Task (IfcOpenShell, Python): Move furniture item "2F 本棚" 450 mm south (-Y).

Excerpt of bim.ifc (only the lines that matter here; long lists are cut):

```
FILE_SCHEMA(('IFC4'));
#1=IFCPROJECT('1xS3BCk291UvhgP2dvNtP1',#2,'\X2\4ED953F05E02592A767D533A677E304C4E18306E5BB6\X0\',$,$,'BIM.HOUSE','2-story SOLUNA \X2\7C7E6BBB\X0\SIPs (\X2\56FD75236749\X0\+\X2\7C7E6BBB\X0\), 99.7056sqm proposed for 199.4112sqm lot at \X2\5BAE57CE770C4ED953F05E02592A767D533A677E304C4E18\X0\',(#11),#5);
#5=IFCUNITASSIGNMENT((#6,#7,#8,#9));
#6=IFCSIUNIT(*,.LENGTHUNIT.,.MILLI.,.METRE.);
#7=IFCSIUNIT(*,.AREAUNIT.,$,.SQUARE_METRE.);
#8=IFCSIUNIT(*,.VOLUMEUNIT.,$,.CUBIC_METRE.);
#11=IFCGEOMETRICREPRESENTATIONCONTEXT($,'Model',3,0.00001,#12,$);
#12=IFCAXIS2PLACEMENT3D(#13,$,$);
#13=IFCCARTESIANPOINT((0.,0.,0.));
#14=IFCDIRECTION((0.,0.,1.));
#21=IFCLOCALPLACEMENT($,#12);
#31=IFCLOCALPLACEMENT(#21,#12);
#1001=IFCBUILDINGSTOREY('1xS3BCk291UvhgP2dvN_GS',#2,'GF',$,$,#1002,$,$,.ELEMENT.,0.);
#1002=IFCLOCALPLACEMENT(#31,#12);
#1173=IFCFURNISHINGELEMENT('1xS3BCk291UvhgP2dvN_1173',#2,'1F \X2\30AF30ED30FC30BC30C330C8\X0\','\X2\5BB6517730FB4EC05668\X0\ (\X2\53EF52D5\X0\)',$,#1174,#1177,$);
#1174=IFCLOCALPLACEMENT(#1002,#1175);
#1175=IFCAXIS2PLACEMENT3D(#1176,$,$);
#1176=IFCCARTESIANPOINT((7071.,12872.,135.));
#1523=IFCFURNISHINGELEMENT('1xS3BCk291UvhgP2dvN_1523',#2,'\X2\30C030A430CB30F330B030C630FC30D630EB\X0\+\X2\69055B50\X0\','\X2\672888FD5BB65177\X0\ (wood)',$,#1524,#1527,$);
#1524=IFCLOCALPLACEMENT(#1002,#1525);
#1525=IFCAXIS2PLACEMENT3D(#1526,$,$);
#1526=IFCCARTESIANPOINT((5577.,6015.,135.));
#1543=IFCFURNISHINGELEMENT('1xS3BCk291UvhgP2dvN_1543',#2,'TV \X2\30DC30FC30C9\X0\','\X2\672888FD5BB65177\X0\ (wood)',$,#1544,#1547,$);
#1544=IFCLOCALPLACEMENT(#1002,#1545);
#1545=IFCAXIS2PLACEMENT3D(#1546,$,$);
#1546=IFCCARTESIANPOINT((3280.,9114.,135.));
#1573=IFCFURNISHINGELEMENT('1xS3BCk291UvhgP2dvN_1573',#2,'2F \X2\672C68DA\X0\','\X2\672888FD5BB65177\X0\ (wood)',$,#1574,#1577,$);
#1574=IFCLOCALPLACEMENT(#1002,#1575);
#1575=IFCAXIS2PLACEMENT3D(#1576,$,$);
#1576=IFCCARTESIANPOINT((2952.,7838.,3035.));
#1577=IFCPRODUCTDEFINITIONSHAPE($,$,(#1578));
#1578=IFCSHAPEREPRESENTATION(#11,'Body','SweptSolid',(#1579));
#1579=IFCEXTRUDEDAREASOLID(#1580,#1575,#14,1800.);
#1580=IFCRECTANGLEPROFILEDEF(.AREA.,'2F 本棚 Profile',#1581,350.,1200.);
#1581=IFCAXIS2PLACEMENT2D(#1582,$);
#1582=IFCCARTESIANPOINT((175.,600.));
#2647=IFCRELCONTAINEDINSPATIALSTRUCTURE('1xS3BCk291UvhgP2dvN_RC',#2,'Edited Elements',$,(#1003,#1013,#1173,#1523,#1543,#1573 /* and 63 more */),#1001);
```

```python
import ifcopenshell
import ifcopenshell.api.geometry
import ifcopenshell.util.placement

model = ifcopenshell.open("bim.ifc")

item = model.by_guid("1xS3BCk291UvhgP2dvN_1573")
matrix = ifcopenshell.util.placement.get_local_placement(item.ObjectPlacement)
matrix[1, 3] -= 450.0
ifcopenshell.api.geometry.edit_object_placement(model, product=item, matrix=matrix, is_si=False)

print(ifcopenshell.util.placement.get_local_placement(item.ObjectPlacement).round(3) + 0.0)

model.write("bim_edited.ifc")
```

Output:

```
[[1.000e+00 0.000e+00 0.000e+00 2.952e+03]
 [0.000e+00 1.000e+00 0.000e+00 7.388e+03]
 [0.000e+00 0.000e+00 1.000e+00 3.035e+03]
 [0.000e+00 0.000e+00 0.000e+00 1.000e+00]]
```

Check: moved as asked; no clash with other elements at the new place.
